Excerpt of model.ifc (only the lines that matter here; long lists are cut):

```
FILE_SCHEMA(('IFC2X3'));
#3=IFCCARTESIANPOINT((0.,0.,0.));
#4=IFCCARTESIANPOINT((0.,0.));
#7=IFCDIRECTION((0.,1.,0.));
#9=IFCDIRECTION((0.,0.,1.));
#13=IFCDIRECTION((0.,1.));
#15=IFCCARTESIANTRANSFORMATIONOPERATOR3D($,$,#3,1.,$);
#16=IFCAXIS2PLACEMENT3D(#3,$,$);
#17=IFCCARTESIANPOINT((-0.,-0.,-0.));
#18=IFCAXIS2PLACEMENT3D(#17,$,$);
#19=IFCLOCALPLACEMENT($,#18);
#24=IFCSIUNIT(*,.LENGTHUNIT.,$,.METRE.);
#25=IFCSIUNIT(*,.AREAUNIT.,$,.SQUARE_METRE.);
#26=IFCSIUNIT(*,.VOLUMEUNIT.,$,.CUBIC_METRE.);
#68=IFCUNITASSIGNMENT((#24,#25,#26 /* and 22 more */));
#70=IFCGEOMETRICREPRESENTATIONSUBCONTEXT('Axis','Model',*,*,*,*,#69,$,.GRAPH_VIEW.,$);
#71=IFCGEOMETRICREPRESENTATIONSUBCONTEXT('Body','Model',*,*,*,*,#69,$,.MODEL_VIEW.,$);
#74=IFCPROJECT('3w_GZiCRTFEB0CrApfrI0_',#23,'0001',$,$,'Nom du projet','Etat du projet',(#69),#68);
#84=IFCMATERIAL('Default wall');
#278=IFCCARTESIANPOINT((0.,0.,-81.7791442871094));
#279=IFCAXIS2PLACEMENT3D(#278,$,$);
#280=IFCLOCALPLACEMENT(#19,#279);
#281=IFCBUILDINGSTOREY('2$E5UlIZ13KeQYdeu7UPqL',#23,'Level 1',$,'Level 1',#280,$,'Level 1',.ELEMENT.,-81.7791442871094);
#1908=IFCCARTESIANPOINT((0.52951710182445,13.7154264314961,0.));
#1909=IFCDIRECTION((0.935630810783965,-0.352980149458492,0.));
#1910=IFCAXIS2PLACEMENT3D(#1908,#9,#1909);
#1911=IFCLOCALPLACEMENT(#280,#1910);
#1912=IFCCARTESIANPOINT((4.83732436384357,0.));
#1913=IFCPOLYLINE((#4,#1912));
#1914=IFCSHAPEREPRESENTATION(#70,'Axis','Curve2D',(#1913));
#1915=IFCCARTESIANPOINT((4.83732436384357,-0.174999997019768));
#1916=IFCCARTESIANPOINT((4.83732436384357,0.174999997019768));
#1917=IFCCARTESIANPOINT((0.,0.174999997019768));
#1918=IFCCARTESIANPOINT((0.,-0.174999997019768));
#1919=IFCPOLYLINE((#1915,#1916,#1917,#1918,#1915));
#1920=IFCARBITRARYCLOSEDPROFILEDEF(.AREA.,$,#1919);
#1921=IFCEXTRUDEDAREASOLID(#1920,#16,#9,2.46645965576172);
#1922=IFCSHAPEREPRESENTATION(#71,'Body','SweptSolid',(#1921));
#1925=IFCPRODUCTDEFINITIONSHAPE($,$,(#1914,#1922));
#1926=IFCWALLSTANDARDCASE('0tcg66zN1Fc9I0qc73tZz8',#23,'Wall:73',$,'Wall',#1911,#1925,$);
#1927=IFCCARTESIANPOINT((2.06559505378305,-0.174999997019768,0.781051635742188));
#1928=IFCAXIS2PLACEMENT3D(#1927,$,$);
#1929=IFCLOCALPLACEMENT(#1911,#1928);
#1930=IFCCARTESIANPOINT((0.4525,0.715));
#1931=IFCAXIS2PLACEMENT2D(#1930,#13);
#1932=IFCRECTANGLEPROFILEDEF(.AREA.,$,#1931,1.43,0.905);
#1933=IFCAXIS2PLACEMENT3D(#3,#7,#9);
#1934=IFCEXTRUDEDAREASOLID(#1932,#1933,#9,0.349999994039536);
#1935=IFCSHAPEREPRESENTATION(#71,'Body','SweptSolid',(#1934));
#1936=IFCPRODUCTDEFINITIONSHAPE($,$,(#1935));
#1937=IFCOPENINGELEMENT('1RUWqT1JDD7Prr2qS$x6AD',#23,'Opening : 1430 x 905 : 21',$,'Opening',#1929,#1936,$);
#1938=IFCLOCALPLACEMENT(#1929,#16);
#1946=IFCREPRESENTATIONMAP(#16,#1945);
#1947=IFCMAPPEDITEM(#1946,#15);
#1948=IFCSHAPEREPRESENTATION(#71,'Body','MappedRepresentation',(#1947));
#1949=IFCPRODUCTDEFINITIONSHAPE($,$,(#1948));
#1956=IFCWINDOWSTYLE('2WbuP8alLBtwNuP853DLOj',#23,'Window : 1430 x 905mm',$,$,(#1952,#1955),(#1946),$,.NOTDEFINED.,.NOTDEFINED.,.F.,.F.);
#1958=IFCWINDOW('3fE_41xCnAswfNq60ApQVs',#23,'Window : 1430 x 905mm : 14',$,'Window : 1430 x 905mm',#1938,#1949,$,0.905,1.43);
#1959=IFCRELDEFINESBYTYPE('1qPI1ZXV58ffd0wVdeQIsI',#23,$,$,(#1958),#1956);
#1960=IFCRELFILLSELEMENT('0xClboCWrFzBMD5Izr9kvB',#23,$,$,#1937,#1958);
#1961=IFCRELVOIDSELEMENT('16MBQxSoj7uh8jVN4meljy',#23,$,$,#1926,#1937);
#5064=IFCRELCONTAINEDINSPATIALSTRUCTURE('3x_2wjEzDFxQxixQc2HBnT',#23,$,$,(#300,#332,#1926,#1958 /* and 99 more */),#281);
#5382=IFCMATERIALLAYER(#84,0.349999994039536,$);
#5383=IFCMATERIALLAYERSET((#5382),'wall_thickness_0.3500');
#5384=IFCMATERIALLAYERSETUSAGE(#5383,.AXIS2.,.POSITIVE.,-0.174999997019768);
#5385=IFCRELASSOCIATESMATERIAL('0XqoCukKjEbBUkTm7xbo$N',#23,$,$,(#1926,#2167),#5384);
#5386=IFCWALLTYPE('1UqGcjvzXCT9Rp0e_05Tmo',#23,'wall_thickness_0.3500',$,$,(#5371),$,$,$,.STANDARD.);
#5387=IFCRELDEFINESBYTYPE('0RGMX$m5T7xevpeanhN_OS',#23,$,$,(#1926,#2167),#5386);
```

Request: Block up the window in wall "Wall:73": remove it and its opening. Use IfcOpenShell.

```python
import ifcopenshell
import ifcopenshell.api.feature
import ifcopenshell.api.root
import ifcopenshell.geom
import ifcopenshell.util.shape

model = ifcopenshell.open("model.ifc")
settings = ifcopenshell.geom.settings()


def volume(element):
    """Net volume in cubic metres, openings subtracted."""
    shape = ifcopenshell.geom.create_shape(settings, element)
    return ifcopenshell.util.shape.get_volume(shape.geometry)


window = model.by_guid("3fE_41xCnAswfNq60ApQVs")
opening = window.FillsVoids[0].RelatingOpeningElement
wall = opening.VoidsElements[0].RelatingBuildingElement
before = volume(wall)

ifcopenshell.api.root.remove_product(model, product=window)
ifcopenshell.api.feature.remove_feature(model, feature=opening)

after = volume(wall)

print(f"wall volume {before:.3f} -> {after:.3f} m3")

model.write("model_v2.ifc")
```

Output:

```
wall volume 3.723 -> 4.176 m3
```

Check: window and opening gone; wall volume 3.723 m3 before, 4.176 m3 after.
